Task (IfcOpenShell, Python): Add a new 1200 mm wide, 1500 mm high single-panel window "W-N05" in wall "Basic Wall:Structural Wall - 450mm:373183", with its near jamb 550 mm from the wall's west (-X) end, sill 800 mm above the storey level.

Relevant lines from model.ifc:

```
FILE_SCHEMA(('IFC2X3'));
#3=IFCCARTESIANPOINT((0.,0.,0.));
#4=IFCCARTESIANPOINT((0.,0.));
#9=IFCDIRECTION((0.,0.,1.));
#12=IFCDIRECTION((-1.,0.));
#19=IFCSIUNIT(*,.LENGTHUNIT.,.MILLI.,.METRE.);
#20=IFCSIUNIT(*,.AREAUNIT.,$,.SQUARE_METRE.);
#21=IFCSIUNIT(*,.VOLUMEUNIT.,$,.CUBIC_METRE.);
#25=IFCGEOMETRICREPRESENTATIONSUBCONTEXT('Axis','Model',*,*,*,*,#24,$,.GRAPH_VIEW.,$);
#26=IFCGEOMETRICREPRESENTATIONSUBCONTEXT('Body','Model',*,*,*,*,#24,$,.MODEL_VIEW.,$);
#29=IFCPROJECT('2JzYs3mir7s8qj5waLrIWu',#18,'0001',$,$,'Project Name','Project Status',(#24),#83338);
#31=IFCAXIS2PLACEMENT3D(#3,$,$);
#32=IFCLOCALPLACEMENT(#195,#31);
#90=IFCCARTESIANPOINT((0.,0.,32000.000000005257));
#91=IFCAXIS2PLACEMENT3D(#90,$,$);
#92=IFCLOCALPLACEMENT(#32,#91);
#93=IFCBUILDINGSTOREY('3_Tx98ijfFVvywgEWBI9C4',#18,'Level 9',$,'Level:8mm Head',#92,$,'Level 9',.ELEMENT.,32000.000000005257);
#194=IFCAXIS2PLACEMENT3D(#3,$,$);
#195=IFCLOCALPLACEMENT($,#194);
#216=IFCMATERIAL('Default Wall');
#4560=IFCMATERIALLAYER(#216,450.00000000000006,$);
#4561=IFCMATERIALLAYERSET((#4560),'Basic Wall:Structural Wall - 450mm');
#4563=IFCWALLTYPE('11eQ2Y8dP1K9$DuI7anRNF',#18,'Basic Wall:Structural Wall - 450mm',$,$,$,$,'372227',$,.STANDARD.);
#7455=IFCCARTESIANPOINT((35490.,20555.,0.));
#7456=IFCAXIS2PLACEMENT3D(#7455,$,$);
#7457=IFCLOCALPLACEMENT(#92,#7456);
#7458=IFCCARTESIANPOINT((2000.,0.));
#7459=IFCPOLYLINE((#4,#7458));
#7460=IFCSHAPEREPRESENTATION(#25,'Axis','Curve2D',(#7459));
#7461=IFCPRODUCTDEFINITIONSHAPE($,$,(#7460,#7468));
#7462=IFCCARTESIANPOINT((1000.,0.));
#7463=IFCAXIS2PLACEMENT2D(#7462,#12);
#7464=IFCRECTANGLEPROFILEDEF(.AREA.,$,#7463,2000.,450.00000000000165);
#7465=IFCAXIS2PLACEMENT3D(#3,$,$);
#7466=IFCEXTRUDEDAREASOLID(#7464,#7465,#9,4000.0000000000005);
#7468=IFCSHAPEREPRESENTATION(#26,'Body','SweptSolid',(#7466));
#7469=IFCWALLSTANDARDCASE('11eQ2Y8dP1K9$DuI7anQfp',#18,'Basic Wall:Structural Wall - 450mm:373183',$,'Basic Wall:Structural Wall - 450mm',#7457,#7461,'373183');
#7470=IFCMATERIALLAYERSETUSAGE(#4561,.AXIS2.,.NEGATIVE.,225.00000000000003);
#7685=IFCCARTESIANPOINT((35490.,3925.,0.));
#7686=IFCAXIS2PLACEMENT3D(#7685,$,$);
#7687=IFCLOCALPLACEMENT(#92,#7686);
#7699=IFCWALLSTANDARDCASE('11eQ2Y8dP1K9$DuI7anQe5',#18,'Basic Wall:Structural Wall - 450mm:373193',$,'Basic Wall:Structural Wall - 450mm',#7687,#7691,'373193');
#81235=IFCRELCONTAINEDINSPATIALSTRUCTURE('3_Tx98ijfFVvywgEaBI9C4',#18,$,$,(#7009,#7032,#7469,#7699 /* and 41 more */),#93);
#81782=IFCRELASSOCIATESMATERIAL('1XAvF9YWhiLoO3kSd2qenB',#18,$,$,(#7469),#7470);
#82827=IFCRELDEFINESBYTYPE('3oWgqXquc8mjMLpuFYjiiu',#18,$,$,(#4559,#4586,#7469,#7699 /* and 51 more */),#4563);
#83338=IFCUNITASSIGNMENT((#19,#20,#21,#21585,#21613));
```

```python
import numpy as np
import ifcopenshell
import ifcopenshell.api.feature
import ifcopenshell.api.geometry
import ifcopenshell.api.root
import ifcopenshell.api.spatial
import ifcopenshell.api.type
import ifcopenshell.geom
import ifcopenshell.util.element
import ifcopenshell.util.placement
import ifcopenshell.util.representation
import ifcopenshell.util.shape
import ifcopenshell.util.unit

model = ifcopenshell.open("model.ifc")
unit_scale = ifcopenshell.util.unit.calculate_unit_scale(model)
settings = ifcopenshell.geom.settings()


def volume(element):
    """Net volume in cubic metres, openings subtracted."""
    shape = ifcopenshell.geom.create_shape(settings, element)
    return ifcopenshell.util.shape.get_volume(shape.geometry)


wall = model.by_guid("11eQ2Y8dP1K9$DuI7anQfp")
storey = ifcopenshell.util.element.get_container(wall, ifc_class="IfcBuildingStorey")
context = ifcopenshell.util.representation.get_context(model, "Model", "Body", "MODEL_VIEW")
before = volume(wall)

width, height, from_end, sill = 1.2, 1.5, 0.55, 0.8  # metres

# The wall runs along its own X axis, and the end named is its -X end.
wall_shape = ifcopenshell.geom.create_shape(settings, wall)
x, y, z = ifcopenshell.util.shape.get_vertices(wall_shape.geometry).T
start = x.min() + from_end
face, thickness = float(y.min()), float(y.max() - y.min())
wall_matrix = ifcopenshell.util.placement.get_local_placement(wall.ObjectPlacement)
level = ifcopenshell.util.placement.get_local_placement(storey.ObjectPlacement)[2, 3]


def in_wall(x, y):
    """Placement at x, y metres in the wall's axes, at sill height."""
    matrix = wall_matrix.copy()
    matrix[:, 3] = wall_matrix @ np.array([x / unit_scale, y / unit_scale, 0.0, 1.0])
    matrix[2, 3] = level + sill / unit_scale
    return matrix


# Opening: a box that overshoots both wall faces by 50 mm.
opening = ifcopenshell.api.root.create_entity(model, ifc_class="IfcOpeningElement")
box = ifcopenshell.api.geometry.add_wall_representation(
    model, context=context, length=width, height=height, thickness=thickness + 0.1
)
ifcopenshell.api.geometry.assign_representation(model, product=opening, representation=box)
ifcopenshell.api.geometry.edit_object_placement(model, product=opening, matrix=in_wall(start, face - 0.05), is_si=False)
ifcopenshell.api.feature.add_feature(model, feature=opening, element=wall)

window = ifcopenshell.api.root.create_entity(model, ifc_class="IfcWindow", name="W-N05")
window.OverallWidth, window.OverallHeight = width / unit_scale, height / unit_scale
body = ifcopenshell.api.geometry.add_window_representation(
    model,
    context=context,
    overall_width=window.OverallWidth,
    overall_height=window.OverallHeight,
    partition_type="SINGLE_PANEL",
)
ifcopenshell.api.geometry.assign_representation(model, product=window, representation=body)
ifcopenshell.api.spatial.assign_container(model, products=[window], relating_structure=storey)
fills = ifcopenshell.api.feature.add_filling(model, opening=opening, element=window)
fills.OwnerHistory = window.OwnerHistory  # required in IFC2X3

# IFC2X3 keeps the operation on the window style.
style = ifcopenshell.api.root.create_entity(model, ifc_class="IfcWindowStyle", name="W-N05")
style.OperationType, style.ConstructionType = "SINGLE_PANEL", "NOTDEFINED"
style.ParameterTakesPrecedence = style.Sizeable = False
ifcopenshell.api.type.assign_type(model, related_objects=[window], relating_type=style)

# Centre the window in the wall's thickness.
ifcopenshell.api.geometry.edit_object_placement(model, product=window, matrix=in_wall(start, face), is_si=False)
window_shape = ifcopenshell.geom.create_shape(settings, window)
depth = ifcopenshell.util.shape.get_vertices(window_shape.geometry)[:, 1]
offset = face + thickness / 2 - (depth.min() + depth.max()) / 2
ifcopenshell.api.geometry.edit_object_placement(model, product=window, matrix=in_wall(start, offset), is_si=False)

after = volume(wall)

print(f"wall volume {before:.3f} -> {after:.3f} m3")

model.write("model_v2.ifc")
```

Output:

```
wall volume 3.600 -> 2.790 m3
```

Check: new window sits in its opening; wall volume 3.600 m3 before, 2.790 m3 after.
